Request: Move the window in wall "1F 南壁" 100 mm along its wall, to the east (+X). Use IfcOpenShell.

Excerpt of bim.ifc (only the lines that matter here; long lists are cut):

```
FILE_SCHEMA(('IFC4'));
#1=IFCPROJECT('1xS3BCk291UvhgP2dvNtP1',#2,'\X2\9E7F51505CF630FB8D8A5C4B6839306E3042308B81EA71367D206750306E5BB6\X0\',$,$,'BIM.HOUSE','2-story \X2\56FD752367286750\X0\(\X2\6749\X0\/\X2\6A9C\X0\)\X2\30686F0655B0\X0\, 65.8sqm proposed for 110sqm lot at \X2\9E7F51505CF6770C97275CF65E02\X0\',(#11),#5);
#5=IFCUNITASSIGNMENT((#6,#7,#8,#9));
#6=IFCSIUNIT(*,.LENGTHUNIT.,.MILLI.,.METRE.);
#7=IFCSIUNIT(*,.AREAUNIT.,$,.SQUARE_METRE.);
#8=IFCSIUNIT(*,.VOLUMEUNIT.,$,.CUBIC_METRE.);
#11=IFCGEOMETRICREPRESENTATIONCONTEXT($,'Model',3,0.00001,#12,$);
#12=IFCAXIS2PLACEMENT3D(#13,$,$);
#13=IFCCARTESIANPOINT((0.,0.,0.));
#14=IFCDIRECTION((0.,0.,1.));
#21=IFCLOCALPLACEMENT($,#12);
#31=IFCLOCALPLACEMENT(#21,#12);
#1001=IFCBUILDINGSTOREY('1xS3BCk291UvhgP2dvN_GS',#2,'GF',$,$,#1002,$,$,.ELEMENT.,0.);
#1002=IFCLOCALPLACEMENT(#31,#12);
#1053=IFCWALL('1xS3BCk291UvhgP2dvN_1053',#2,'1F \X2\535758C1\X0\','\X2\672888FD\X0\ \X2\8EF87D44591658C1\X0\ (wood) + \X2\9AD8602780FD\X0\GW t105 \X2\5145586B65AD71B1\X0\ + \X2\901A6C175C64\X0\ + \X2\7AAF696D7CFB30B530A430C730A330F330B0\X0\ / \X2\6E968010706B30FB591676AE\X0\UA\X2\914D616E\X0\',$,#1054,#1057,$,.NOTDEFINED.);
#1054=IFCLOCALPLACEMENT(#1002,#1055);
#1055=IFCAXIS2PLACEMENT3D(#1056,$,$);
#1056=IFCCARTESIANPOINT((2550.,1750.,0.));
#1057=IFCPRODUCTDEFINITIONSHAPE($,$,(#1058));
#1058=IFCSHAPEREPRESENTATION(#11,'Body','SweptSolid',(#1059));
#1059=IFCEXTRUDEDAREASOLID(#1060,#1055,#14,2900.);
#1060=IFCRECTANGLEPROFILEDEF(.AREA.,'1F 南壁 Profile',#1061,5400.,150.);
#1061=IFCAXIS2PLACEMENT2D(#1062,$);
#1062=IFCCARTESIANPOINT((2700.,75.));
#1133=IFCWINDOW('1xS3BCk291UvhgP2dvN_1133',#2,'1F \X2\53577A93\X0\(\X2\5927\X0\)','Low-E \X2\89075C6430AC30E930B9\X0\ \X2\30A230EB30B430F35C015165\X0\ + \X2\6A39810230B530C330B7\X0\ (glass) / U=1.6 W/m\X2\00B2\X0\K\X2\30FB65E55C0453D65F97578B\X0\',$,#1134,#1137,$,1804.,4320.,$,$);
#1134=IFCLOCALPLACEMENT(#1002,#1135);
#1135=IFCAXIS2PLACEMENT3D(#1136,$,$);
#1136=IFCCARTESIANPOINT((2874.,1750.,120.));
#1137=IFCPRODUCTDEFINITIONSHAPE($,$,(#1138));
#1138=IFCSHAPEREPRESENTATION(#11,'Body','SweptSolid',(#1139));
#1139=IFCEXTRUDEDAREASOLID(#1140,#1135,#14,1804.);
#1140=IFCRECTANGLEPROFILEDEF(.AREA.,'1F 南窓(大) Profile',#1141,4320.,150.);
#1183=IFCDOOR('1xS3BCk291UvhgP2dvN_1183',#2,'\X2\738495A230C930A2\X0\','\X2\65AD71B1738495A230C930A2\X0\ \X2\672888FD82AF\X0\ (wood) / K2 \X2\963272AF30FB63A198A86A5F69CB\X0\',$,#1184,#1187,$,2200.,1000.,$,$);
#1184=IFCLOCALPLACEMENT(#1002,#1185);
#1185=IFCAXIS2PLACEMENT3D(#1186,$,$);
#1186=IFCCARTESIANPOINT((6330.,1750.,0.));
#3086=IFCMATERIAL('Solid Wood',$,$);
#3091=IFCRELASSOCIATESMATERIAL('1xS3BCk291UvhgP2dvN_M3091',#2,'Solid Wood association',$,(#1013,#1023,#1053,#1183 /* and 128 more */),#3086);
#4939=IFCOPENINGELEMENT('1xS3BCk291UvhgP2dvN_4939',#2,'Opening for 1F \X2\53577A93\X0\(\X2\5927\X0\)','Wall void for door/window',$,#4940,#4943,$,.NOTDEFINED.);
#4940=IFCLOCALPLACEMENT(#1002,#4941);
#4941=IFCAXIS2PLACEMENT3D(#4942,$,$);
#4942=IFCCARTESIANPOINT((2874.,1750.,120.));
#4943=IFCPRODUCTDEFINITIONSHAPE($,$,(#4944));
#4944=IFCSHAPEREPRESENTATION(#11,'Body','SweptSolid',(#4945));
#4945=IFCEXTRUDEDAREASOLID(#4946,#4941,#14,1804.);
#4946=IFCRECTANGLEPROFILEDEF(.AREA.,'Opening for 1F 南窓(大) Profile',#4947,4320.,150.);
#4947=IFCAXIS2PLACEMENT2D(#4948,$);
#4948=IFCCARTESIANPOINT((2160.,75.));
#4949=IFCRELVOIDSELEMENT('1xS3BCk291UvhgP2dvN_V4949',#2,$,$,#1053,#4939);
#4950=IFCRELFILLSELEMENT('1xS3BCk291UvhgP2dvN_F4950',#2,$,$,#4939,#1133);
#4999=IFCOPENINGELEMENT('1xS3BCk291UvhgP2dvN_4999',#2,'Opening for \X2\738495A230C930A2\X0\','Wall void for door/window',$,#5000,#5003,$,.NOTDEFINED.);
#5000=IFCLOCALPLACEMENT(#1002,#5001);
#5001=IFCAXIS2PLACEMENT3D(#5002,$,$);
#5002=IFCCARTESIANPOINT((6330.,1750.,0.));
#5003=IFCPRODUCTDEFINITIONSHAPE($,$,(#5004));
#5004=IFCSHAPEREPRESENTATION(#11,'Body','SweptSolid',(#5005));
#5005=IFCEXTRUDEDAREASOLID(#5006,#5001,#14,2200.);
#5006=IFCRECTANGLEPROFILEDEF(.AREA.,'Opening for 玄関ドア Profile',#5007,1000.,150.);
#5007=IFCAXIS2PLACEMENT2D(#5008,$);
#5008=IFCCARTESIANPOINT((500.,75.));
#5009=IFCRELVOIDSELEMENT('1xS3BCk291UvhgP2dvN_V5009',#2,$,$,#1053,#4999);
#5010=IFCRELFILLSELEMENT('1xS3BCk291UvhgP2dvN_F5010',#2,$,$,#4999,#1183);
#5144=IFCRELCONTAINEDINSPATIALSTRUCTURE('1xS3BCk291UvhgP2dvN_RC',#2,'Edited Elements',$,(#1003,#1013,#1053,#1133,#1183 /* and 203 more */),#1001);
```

```python
import ifcopenshell
import ifcopenshell.api.geometry
import ifcopenshell.util.placement

model = ifcopenshell.open("bim.ifc")

window = model.by_id(1133)
opening = window.FillsVoids[0].RelatingOpeningElement
wall = opening.VoidsElements[0].RelatingBuildingElement

wall_matrix = ifcopenshell.util.placement.get_local_placement(wall.ObjectPlacement)
shift = wall_matrix[:3, 0] * 100.0
before = ifcopenshell.util.placement.get_local_placement(window.ObjectPlacement)[:3, 3].copy()

# The window is not placed relative to its opening, so move both.
for product in (opening, window):
    matrix = ifcopenshell.util.placement.get_local_placement(product.ObjectPlacement)
    matrix[:3, 3] += shift
    ifcopenshell.api.geometry.edit_object_placement(model, product=product, matrix=matrix, is_si=False)

after = ifcopenshell.util.placement.get_local_placement(window.ObjectPlacement)[:3, 3]
print("window moved by", (after - before).round(3) + 0.0)

model.write("bim-out.ifc")
```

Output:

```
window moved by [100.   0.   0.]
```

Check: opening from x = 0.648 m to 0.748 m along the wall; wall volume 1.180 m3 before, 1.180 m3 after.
